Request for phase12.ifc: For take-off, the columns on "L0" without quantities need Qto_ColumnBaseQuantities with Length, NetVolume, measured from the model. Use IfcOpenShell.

First a look at what the model holds.

```python
import ifcopenshell
import ifcopenshell.util.element
import ifcopenshell.util.unit

model = ifcopenshell.open("phase12.ifc")
print(model.schema)
for unit_type in ("LENGTHUNIT", "AREAUNIT", "VOLUMEUNIT"):
    print(unit_type, ifcopenshell.util.unit.calculate_unit_scale(model, unit_type))
storey = next(s for s in model.by_type("IfcBuildingStorey") if s.Name == "L0")
columns = [e for e in ifcopenshell.util.element.get_decomposition(storey) if e.is_a("IfcColumn")]
for e in sorted(columns, key=lambda e: e.id()):
    print(e.id(), e.is_a(), e.Name, list(ifcopenshell.util.element.get_psets(e, qtos_only=True)), sep=" | ")
```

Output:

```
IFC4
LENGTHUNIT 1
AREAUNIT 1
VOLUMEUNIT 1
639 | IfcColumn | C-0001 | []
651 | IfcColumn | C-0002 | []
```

```python
import ifcopenshell
import ifcopenshell.api.pset
import ifcopenshell.geom
import ifcopenshell.util.element
import ifcopenshell.util.shape
import ifcopenshell.util.unit

model = ifcopenshell.open("phase12.ifc")
unit_scale = ifcopenshell.util.unit.calculate_unit_scale(model)
volume_scale = ifcopenshell.util.unit.calculate_unit_scale(model, "VOLUMEUNIT")
settings = ifcopenshell.geom.settings()

storey = next(s for s in model.by_type("IfcBuildingStorey") if s.Name == "L0")
columns = [e for e in ifcopenshell.util.element.get_decomposition(storey) if e.is_a("IfcColumn")]

for e in sorted(columns, key=lambda e: e.id()):
    if ifcopenshell.util.element.get_psets(e, qtos_only=True, should_inherit=False):
        continue
    # Geometry comes back in metres, in the element's own axes.
    shape = ifcopenshell.geom.create_shape(settings, e)
    values = {
        "Length": ifcopenshell.util.shape.get_z(shape.geometry) / unit_scale,
        "NetVolume": ifcopenshell.util.shape.get_volume(shape.geometry) / volume_scale,
    }
    qto = ifcopenshell.api.pset.add_qto(model, product=e, name="Qto_ColumnBaseQuantities")
    ifcopenshell.api.pset.edit_qto(model, qto=qto, properties=values)
    print(e.id(), {k: round(v, 3) for k, v in values.items()})

model.write("phase12_v2.ifc")
```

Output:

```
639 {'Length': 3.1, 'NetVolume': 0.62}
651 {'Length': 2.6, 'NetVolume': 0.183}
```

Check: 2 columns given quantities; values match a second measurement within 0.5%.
